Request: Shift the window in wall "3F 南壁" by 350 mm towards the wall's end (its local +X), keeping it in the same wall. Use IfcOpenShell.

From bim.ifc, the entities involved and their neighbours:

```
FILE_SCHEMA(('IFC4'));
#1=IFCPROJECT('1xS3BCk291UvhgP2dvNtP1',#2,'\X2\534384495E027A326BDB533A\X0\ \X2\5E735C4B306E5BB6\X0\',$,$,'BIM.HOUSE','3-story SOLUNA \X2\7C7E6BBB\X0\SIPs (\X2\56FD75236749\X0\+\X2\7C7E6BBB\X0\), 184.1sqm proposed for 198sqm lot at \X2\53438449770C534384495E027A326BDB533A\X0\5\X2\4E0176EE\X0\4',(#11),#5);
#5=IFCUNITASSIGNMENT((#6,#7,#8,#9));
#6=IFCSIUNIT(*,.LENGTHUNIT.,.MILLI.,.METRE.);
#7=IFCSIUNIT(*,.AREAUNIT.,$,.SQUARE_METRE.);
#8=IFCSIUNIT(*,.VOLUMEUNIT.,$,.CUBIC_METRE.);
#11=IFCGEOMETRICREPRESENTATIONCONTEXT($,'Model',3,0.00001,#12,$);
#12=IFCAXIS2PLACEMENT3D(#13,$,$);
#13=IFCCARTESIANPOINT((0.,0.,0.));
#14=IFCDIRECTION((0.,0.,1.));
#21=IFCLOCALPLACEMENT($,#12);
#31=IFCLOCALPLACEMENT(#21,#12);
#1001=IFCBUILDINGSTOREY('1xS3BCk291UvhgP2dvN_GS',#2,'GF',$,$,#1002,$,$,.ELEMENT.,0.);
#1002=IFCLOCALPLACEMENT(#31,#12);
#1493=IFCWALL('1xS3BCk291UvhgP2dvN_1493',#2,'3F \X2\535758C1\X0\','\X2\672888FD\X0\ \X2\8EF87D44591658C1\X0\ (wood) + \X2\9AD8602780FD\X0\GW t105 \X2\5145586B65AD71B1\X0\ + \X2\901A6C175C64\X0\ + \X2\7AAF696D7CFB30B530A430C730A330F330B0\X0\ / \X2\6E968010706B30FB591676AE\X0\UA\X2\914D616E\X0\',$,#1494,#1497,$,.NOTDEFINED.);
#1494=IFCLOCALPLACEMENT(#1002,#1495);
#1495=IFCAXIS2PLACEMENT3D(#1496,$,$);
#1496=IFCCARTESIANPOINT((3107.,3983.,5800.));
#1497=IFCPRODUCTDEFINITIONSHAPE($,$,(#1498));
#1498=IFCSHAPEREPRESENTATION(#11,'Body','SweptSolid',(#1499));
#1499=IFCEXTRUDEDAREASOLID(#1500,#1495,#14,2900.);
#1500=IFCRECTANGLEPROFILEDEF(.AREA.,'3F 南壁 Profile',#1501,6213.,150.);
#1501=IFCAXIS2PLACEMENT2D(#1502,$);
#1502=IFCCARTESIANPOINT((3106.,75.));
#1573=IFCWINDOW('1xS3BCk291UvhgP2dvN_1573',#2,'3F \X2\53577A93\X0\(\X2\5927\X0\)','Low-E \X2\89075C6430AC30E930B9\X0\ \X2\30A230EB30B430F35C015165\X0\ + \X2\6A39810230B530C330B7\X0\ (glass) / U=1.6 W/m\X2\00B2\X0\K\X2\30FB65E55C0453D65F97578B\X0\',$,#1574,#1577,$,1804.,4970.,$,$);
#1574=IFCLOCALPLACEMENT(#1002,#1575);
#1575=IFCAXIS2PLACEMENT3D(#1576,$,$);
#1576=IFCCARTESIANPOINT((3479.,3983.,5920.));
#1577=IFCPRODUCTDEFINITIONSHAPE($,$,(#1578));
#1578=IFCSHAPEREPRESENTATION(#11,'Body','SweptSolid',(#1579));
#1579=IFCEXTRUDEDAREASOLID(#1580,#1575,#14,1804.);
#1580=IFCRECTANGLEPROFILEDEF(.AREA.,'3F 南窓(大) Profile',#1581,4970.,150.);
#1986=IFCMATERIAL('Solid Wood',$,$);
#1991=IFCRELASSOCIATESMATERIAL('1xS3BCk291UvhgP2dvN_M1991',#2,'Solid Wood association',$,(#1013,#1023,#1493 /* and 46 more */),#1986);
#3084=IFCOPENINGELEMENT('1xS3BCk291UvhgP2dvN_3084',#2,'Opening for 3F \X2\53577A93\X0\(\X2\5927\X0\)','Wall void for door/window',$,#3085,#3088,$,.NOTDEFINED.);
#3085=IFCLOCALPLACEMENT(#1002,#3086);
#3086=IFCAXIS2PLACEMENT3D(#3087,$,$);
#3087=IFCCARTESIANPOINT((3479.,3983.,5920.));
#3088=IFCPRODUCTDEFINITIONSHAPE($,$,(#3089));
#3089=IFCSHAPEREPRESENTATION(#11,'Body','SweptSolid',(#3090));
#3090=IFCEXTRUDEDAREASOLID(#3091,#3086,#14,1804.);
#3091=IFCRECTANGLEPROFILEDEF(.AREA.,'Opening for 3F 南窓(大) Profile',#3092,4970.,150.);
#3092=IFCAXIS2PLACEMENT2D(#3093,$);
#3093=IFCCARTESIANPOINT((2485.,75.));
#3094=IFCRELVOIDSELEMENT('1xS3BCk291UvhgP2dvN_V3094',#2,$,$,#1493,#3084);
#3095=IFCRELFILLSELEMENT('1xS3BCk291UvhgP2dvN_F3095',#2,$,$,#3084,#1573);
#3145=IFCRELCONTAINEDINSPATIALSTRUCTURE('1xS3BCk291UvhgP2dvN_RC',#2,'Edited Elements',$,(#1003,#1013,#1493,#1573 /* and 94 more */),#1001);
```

```python
import ifcopenshell
import ifcopenshell.api.geometry
import ifcopenshell.util.placement
import ifcopenshell.util.unit

model = ifcopenshell.open("bim.ifc")
unit_scale = ifcopenshell.util.unit.calculate_unit_scale(model)

window = model.by_guid("1xS3BCk291UvhgP2dvN_1573")
opening = window.FillsVoids[0].RelatingOpeningElement
wall = opening.VoidsElements[0].RelatingBuildingElement

wall_matrix = ifcopenshell.util.placement.get_local_placement(wall.ObjectPlacement)
shift = wall_matrix[:3, 0] * 0.35 / unit_scale
before = ifcopenshell.util.placement.get_local_placement(window.ObjectPlacement)[:3, 3].copy()

# The window is not placed relative to its opening, so move both.
for product in (opening, window):
    matrix = ifcopenshell.util.placement.get_local_placement(product.ObjectPlacement)
    matrix[:3, 3] += shift
    ifcopenshell.api.geometry.edit_object_placement(model, product=product, matrix=matrix, is_si=False)

after = ifcopenshell.util.placement.get_local_placement(window.ObjectPlacement)[:3, 3]
print("window moved by", (after - before).round(3) + 0.0)

model.write("bim_edited.ifc")
```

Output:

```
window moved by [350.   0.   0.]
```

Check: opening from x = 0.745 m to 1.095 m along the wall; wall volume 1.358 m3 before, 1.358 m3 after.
